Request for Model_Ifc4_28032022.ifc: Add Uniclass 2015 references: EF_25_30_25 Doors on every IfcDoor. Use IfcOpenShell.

First a look at what the model holds.

```python
import ifcopenshell

model = ifcopenshell.open("Model_Ifc4_28032022.ifc")
print(model.schema)
print("classifications:", [c.Name for c in model.by_type("IfcClassification")])
for ifc_class in ("IfcDoor", "IfcRoof", "IfcStair", "IfcWall", "IfcWindow"):
    print(ifc_class, len(model.by_type(ifc_class)))
```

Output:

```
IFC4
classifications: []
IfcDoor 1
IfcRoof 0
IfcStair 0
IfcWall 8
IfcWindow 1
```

```python
import ifcopenshell
import ifcopenshell.api.classification

model = ifcopenshell.open("Model_Ifc4_28032022.ifc")

system = ifcopenshell.api.classification.add_classification(model, classification="Uniclass 2015")

codes = {
    "IfcDoor": ("EF_25_30_25", "Doors"),
}
for ifc_class, (code, name) in codes.items():
    products = model.by_type(ifc_class)
    ifcopenshell.api.classification.add_reference(
        model, products=products, classification=system, identification=code, name=name
    )
    print(code, len(products))

model.write("Model_Ifc4_28032022_v2.ifc")
```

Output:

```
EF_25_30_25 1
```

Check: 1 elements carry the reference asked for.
